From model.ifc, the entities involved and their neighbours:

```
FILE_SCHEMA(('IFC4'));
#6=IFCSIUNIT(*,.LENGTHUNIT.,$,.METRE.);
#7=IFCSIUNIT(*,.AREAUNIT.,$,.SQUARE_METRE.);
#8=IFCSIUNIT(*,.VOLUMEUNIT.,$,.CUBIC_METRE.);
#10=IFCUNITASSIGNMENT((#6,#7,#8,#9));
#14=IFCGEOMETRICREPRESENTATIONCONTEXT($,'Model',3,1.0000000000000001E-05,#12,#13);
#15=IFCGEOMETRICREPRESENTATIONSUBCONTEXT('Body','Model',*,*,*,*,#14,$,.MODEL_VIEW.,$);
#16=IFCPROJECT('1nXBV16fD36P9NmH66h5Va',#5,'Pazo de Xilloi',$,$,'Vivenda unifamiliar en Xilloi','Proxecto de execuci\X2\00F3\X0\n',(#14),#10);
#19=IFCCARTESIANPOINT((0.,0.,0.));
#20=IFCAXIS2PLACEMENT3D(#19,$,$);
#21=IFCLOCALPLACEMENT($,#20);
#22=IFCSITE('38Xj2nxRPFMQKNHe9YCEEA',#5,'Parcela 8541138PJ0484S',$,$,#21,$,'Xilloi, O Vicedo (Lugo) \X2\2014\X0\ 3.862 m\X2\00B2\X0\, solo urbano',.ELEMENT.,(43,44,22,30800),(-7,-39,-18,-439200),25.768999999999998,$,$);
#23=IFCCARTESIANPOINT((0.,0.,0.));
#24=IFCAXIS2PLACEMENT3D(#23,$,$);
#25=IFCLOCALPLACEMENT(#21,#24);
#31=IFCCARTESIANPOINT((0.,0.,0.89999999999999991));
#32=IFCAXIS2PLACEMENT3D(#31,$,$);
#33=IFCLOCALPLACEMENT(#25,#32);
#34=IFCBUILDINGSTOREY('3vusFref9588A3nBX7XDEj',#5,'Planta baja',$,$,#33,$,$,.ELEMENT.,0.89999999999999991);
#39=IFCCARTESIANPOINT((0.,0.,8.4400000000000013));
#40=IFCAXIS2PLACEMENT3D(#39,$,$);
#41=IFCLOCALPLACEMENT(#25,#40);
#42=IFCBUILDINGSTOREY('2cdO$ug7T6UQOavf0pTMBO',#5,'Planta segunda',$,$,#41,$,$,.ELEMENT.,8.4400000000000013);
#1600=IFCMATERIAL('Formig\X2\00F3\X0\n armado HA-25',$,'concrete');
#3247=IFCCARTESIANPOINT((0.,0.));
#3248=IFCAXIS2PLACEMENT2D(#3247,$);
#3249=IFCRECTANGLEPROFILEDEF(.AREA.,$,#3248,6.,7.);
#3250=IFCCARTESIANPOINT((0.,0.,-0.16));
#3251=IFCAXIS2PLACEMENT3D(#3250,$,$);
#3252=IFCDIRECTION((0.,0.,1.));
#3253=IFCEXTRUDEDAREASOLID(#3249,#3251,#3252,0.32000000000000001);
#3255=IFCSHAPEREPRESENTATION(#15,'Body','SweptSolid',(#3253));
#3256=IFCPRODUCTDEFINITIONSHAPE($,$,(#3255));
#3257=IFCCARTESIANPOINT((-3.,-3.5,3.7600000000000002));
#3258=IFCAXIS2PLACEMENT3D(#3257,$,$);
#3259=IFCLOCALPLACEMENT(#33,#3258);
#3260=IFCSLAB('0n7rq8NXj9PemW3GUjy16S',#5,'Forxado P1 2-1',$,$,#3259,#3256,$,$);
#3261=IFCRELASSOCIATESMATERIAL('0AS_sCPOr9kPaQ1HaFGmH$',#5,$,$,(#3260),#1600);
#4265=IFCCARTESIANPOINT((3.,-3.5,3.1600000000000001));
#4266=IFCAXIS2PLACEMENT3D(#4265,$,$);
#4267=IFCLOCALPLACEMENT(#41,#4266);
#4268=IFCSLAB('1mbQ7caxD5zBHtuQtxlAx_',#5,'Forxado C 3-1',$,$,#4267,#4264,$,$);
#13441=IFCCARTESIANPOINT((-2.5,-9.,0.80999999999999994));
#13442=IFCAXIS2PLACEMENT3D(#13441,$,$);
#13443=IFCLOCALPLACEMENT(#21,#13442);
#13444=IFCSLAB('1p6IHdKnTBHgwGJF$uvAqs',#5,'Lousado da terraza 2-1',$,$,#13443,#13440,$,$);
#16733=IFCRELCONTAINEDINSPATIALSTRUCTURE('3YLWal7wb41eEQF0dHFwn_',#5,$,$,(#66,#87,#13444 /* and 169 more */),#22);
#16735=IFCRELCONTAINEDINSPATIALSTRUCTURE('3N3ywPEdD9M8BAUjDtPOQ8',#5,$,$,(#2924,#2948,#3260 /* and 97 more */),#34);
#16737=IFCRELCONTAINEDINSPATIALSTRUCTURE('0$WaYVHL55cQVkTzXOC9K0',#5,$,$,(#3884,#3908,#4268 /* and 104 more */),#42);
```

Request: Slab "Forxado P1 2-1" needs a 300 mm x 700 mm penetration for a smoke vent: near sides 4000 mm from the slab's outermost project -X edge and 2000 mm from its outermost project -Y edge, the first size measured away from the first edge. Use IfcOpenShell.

```python
import numpy as np
import ifcopenshell
import ifcopenshell.api.feature
import ifcopenshell.api.geometry
import ifcopenshell.api.root
import ifcopenshell.geom
import ifcopenshell.util.placement
import ifcopenshell.util.representation
import ifcopenshell.util.shape
import ifcopenshell.util.unit

model = ifcopenshell.open("model.ifc")
unit_scale = ifcopenshell.util.unit.calculate_unit_scale(model)
settings = ifcopenshell.geom.settings()


def volume(element):
    """Net volume in cubic metres, openings subtracted."""
    shape = ifcopenshell.geom.create_shape(settings, element)
    return ifcopenshell.util.shape.get_volume(shape.geometry)


slab = model.by_guid("0n7rq8NXj9PemW3GUjy16S")
before = volume(slab)

# Extent in the slab's own axes, in metres. The edges named are its -X and -Y sides.
slab_shape = ifcopenshell.geom.create_shape(settings, slab)
vertices = ifcopenshell.util.shape.get_vertices(slab_shape.geometry)
x_min, y_min, bottom = vertices.min(axis=0)
top = vertices[:, 2].max()

opening = ifcopenshell.api.root.create_entity(model, ifc_class="IfcOpeningElement", name="Smoke vent opening", predefined_type="OPENING")
context = ifcopenshell.util.representation.get_context(model, "Model", "Body", "MODEL_VIEW")
width, depth = 0.3, 0.7
outline = [(0.0, 0.0), (width, 0.0), (width, depth), (0.0, depth), (0.0, 0.0)]
# Overshoot both faces by 50 mm so the cut is clean.
shape = ifcopenshell.api.geometry.add_slab_representation(
    model, context=context, depth=top - bottom + 0.1, polyline=outline
)
ifcopenshell.api.geometry.assign_representation(model, product=opening, representation=shape)

matrix = ifcopenshell.util.placement.get_local_placement(slab.ObjectPlacement)
matrix[:, 3] = matrix @ np.append(np.array([x_min + 4, y_min + 2, bottom - 0.05]) / unit_scale, 1.0)
ifcopenshell.api.geometry.edit_object_placement(model, product=opening, matrix=matrix, is_si=False)
ifcopenshell.api.feature.add_feature(model, feature=opening, element=slab)

after = volume(slab)

print(f"slab volume {before:.3f} -> {after:.3f} m3")

model.write("model-out.ifc")
```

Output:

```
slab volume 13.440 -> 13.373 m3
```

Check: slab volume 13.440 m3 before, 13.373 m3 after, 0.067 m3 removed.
